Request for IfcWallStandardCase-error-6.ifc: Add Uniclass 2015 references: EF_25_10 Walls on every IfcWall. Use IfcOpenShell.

First a look at what the model holds.

```python
import ifcopenshell

model = ifcopenshell.open("IfcWallStandardCase-error-6.ifc")
print(model.schema)
print("classifications:", [c.Name for c in model.by_type("IfcClassification")])
for ifc_class in ("IfcDoor", "IfcRoof", "IfcStair", "IfcWall", "IfcWindow"):
    print(ifc_class, len(model.by_type(ifc_class)))
```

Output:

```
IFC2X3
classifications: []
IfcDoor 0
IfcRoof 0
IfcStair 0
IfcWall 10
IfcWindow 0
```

```python
import ifcopenshell
import ifcopenshell.api.classification

model = ifcopenshell.open("IfcWallStandardCase-error-6.ifc")

# IFC2X3 requires Source and Edition and has no link from the project to the system.
system = model.create_entity("IfcClassification", Source="NBS", Edition="2015", Name="Uniclass 2015")

codes = {
    "IfcWall": ("EF_25_10", "Walls"),
}
for ifc_class, (code, name) in codes.items():
    products = model.by_type(ifc_class)
    ifcopenshell.api.classification.add_reference(
        model, products=products, classification=system, identification=code, name=name
    )
    print(code, len(products))

model.write("IfcWallStandardCase-error-6_rev.ifc")
```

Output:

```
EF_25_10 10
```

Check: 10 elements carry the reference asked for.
